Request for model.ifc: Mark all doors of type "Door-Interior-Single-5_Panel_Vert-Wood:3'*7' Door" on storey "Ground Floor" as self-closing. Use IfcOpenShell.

First a look at what the model holds.

```python
import ifcopenshell
import ifcopenshell.util.element

model = ifcopenshell.open("model.ifc")
print(model.schema)
storey = next(s for s in model.by_type("IfcBuildingStorey") if s.Name == "Ground Floor")
doors = [e for e in ifcopenshell.util.element.get_decomposition(storey) if e.is_a("IfcDoor")]
seen = {}
for e in doors:
    element_type = ifcopenshell.util.element.get_type(e)
    key = (element_type.Name if element_type != e and element_type else None, ifcopenshell.util.element.get_pset(e, "Pset_DoorCommon", "SelfClosing"))
    seen[key] = seen.get(key, 0) + 1
for (name, value), count in sorted(seen.items(), key=str):
    print(count, "x", name, "|", value)
```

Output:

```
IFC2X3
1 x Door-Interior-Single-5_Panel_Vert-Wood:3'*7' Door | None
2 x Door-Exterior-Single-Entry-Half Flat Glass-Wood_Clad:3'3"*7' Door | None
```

```python
import ifcopenshell
import ifcopenshell.api.pset
import ifcopenshell.util.element

model = ifcopenshell.open("model.ifc")

storey = next(s for s in model.by_type("IfcBuildingStorey") if s.Name == "Ground Floor")
doors = [e for e in ifcopenshell.util.element.get_decomposition(storey) if e.is_a("IfcDoor")]

count = 0
for e in doors:
    element_type = ifcopenshell.util.element.get_type(e)
    if element_type in (None, e) or element_type.Name != "Door-Interior-Single-5_Panel_Vert-Wood:3'*7' Door":
        continue
    # add_pset returns the element's existing set when there is one.
    pset = ifcopenshell.api.pset.add_pset(model, product=e, name="Pset_DoorCommon")
    ifcopenshell.api.pset.edit_pset(model, pset=pset, properties={"SelfClosing": True})
    count += 1

print(count, "doors updated")

model.write("model-out.ifc")
```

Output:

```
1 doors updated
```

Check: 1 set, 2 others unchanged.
